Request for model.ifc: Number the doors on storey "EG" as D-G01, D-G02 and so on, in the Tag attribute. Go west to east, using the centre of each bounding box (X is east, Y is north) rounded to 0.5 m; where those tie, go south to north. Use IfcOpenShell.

First a look at what the model holds.

```python
import ifcopenshell
import ifcopenshell.util.element
import ifcopenshell.util.placement

model = ifcopenshell.open("model.ifc")
print(model.schema)
storey = next(s for s in model.by_type("IfcBuildingStorey") if s.Name == "EG")
doors = [e for e in ifcopenshell.util.element.get_decomposition(storey) if e.is_a("IfcDoor")]
for e in sorted(doors, key=lambda e: e.id()):
    origin = ifcopenshell.util.placement.get_local_placement(e.ObjectPlacement)[:3, 3]
    print(e.id(), e.Tag, e.Name, origin.round(2) + 0.0, sep=" | ")
```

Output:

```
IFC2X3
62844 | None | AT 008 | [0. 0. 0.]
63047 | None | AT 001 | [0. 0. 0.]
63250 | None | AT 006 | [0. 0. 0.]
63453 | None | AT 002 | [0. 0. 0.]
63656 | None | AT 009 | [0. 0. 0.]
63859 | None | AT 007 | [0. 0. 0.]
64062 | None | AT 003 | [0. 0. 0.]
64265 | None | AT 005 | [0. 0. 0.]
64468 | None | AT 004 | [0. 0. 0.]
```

```python
import ifcopenshell
import ifcopenshell.geom
import ifcopenshell.util.element
import ifcopenshell.util.shape

model = ifcopenshell.open("model.ifc")
settings = ifcopenshell.geom.settings()
settings.set("use-world-coords", True)


def centre(element):
    shape = ifcopenshell.geom.create_shape(settings, element)
    return ifcopenshell.util.shape.get_bbox_centroid(shape.geometry)


storey = next(s for s in model.by_type("IfcBuildingStorey") if s.Name == "EG")
doors = [e for e in ifcopenshell.util.element.get_decomposition(storey) if e.is_a("IfcDoor")]

# Insertion points can sit at a corner or the storey origin, so sort by the geometry (in metres).
centres = {e: centre(e) for e in doors}
doors.sort(key=lambda e: (round(centres[e][0] / 0.5), centres[e][1]))

for i, e in enumerate(doors, start=1):
    number = f"D-G{i:02d}"
    e.Tag = number
    print(e.id(), number)

model.write("model_edited.ifc")
```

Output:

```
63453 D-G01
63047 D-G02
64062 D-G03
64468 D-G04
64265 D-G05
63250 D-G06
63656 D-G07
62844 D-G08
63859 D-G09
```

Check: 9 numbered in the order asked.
